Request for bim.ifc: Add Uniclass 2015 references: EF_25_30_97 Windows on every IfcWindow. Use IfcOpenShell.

First a look at what the model holds.

```python
import ifcopenshell

model = ifcopenshell.open("bim.ifc")
print(model.schema)
print("classifications:", [c.Name for c in model.by_type("IfcClassification")])
for ifc_class in ("IfcDoor", "IfcRoof", "IfcStair", "IfcWall", "IfcWindow"):
    print(ifc_class, len(model.by_type(ifc_class)))
```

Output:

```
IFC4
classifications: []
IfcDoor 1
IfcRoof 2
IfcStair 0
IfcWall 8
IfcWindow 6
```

```python
import ifcopenshell
import ifcopenshell.api.classification

model = ifcopenshell.open("bim.ifc")

system = ifcopenshell.api.classification.add_classification(model, classification="Uniclass 2015")

codes = {
    "IfcWindow": ("EF_25_30_97", "Windows"),
}
for ifc_class, (code, name) in codes.items():
    products = model.by_type(ifc_class)
    ifcopenshell.api.classification.add_reference(
        model, products=products, classification=system, identification=code, name=name
    )
    print(code, len(products))

model.write("bim_rev.ifc")
```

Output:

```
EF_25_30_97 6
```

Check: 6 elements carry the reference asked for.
